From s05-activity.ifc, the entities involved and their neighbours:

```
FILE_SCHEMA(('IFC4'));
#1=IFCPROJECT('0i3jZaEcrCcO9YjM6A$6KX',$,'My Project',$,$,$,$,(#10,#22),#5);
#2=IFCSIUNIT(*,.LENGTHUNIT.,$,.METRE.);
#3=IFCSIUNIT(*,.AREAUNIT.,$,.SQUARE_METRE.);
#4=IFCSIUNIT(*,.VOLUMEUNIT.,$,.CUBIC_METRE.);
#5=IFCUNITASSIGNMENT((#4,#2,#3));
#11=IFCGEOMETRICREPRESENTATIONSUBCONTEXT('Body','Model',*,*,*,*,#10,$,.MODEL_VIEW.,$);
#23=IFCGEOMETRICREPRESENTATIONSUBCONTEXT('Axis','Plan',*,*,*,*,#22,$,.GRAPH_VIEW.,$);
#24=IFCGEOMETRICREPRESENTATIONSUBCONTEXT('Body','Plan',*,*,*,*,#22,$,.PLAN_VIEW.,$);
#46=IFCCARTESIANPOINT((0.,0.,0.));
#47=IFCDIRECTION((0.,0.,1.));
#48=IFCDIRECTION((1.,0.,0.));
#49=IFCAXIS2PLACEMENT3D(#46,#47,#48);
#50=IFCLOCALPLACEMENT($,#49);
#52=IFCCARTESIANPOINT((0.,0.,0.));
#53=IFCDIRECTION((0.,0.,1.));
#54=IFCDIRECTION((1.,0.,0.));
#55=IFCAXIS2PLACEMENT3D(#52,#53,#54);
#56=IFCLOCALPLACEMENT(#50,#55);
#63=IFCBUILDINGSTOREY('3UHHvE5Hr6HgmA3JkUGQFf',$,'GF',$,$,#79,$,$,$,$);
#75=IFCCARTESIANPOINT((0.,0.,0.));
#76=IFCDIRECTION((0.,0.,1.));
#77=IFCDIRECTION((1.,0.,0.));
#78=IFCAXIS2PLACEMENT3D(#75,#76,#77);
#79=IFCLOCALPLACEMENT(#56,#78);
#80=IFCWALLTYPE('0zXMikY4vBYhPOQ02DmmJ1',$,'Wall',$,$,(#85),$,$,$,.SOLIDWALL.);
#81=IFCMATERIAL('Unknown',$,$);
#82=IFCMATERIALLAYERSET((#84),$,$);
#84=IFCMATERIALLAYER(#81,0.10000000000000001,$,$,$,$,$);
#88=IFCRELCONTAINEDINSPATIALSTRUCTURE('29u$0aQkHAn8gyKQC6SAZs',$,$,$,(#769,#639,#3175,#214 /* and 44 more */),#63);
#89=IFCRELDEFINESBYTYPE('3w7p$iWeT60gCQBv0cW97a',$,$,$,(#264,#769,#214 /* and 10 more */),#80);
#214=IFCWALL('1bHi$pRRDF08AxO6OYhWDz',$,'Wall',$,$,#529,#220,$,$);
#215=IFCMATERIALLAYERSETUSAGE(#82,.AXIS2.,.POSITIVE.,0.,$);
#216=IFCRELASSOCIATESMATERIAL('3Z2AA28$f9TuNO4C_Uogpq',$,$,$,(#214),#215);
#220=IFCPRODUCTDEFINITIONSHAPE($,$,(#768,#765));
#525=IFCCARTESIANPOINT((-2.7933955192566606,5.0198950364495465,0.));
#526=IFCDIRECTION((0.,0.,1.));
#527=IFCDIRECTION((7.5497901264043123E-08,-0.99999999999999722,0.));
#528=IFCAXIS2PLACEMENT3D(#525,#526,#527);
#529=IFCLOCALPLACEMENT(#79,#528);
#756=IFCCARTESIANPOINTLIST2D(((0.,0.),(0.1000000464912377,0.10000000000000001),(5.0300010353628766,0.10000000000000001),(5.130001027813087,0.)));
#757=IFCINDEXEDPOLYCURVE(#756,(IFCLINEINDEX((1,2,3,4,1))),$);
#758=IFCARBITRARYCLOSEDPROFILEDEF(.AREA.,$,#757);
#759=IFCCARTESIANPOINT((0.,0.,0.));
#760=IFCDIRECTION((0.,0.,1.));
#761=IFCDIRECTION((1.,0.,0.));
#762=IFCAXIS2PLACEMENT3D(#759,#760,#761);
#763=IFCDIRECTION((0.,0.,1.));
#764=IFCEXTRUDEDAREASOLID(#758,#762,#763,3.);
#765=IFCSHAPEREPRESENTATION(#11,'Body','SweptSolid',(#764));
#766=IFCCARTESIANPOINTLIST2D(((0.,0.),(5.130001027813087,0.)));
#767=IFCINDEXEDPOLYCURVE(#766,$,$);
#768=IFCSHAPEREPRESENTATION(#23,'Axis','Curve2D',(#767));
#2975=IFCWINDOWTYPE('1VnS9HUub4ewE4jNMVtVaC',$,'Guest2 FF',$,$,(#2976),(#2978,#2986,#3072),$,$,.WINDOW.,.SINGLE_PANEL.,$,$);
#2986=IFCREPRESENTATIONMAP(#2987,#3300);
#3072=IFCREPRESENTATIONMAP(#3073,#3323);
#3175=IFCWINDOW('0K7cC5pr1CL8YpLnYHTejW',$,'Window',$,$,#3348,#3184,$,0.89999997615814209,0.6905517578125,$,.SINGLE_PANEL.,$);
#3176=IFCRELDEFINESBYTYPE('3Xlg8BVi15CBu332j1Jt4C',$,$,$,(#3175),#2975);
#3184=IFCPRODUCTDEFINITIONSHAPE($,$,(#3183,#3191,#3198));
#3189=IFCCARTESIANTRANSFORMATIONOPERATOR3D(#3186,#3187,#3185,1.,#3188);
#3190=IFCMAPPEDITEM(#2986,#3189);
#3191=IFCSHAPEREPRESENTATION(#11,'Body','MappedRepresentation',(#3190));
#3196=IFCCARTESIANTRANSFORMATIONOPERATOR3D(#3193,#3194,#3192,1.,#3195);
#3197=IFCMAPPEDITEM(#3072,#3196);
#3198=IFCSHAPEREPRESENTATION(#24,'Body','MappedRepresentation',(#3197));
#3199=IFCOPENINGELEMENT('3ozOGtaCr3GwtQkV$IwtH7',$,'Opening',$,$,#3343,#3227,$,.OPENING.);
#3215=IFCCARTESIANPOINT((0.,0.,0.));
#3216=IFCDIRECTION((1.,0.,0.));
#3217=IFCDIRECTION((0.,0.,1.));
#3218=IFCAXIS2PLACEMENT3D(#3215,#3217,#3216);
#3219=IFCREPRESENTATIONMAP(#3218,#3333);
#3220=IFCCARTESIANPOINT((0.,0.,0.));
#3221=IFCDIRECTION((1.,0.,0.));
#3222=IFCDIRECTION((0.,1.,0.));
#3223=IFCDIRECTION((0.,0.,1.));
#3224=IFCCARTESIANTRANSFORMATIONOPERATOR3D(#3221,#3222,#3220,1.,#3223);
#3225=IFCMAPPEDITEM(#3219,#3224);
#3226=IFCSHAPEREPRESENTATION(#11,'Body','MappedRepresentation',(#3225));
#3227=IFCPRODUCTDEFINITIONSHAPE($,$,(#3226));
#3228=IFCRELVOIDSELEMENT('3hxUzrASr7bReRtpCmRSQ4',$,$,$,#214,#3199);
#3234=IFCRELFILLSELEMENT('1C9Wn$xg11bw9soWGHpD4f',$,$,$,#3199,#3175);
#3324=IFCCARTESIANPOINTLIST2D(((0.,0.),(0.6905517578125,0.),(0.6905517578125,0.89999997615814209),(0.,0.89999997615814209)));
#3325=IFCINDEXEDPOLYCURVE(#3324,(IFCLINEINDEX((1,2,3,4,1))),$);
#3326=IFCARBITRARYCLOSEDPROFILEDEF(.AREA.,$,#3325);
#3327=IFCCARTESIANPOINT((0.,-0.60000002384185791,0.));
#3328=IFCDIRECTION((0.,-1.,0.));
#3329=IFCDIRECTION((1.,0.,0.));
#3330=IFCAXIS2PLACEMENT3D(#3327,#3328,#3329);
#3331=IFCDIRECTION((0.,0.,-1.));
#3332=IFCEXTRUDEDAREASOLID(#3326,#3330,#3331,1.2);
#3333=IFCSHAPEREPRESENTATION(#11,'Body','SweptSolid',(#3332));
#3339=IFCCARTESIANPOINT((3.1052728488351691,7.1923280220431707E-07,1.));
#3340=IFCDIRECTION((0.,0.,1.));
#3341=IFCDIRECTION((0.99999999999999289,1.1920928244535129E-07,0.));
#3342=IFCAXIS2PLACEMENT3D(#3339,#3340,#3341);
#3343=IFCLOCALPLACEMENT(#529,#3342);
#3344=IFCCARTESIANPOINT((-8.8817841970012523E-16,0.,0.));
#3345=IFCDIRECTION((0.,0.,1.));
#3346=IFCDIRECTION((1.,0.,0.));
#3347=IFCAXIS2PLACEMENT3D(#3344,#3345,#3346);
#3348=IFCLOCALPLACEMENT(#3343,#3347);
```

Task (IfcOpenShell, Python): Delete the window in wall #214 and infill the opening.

```python
import ifcopenshell
import ifcopenshell.api.feature
import ifcopenshell.api.root
import ifcopenshell.geom
import ifcopenshell.util.shape

model = ifcopenshell.open("s05-activity.ifc")
settings = ifcopenshell.geom.settings()


def volume(element):
    """Net volume in cubic metres, openings subtracted."""
    shape = ifcopenshell.geom.create_shape(settings, element)
    return ifcopenshell.util.shape.get_volume(shape.geometry)


window = model.by_guid("0K7cC5pr1CL8YpLnYHTejW")
opening = window.FillsVoids[0].RelatingOpeningElement
wall = opening.VoidsElements[0].RelatingBuildingElement
before = volume(wall)

ifcopenshell.api.root.remove_product(model, product=window)
ifcopenshell.api.feature.remove_feature(model, feature=opening)

after = volume(wall)

print(f"wall volume {before:.3f} -> {after:.3f} m3")

model.write("s05-activity_rev.ifc")
```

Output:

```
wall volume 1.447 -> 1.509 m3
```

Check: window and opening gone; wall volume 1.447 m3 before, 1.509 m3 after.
